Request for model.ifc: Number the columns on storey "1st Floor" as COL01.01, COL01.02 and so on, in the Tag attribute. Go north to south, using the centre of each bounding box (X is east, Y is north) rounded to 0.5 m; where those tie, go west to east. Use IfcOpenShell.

First a look at what the model holds.

```python
import ifcopenshell
import ifcopenshell.util.element
import ifcopenshell.util.placement

model = ifcopenshell.open("model.ifc")
print(model.schema)
storey = next(s for s in model.by_type("IfcBuildingStorey") if s.Name == "1st Floor")
columns = [e for e in ifcopenshell.util.element.get_decomposition(storey) if e.is_a("IfcColumn")]
for e in sorted(columns, key=lambda e: e.id()):
    origin = ifcopenshell.util.placement.get_local_placement(e.ObjectPlacement)[:3, 3]
    print(e.id(), e.Tag, e.Name, origin.round(2) + 0.0, sep=" | ")
```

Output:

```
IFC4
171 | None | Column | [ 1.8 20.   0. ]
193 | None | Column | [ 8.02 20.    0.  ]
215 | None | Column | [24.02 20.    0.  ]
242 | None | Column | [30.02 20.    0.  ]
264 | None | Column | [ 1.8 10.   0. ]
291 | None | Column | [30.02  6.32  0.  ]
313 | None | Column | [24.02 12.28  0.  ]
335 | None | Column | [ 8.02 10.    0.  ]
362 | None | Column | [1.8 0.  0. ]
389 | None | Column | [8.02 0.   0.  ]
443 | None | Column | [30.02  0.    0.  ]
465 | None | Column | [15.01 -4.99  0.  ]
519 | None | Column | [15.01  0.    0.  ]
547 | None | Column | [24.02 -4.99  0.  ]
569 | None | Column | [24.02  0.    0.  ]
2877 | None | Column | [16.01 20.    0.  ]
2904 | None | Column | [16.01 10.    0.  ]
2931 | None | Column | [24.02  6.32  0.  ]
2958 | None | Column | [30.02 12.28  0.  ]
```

```python
import ifcopenshell
import ifcopenshell.geom
import ifcopenshell.util.element
import ifcopenshell.util.shape

model = ifcopenshell.open("model.ifc")
settings = ifcopenshell.geom.settings()
settings.set("use-world-coords", True)


def centre(element):
    shape = ifcopenshell.geom.create_shape(settings, element)
    return ifcopenshell.util.shape.get_bbox_centroid(shape.geometry)


storey = next(s for s in model.by_type("IfcBuildingStorey") if s.Name == "1st Floor")
columns = [e for e in ifcopenshell.util.element.get_decomposition(storey) if e.is_a("IfcColumn")]

# Insertion points can sit at a corner or the storey origin, so sort by the geometry (in metres).
centres = {e: centre(e) for e in columns}
columns.sort(key=lambda e: (-round(centres[e][1] / 0.5), centres[e][0]))

for i, e in enumerate(columns, start=1):
    number = f"COL01.{i:02d}"
    e.Tag = number
    print(e.id(), number)

model.write("model-out.ifc")
```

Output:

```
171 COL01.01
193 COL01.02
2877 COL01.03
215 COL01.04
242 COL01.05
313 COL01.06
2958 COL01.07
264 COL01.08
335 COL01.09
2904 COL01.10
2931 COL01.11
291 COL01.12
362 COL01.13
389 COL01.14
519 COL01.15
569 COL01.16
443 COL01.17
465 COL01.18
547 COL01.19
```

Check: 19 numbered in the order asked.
